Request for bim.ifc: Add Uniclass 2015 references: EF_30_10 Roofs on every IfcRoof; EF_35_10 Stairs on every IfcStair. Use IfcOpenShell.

First a look at what the model holds.

```python
import ifcopenshell

model = ifcopenshell.open("bim.ifc")
print(model.schema)
print("classifications:", [c.Name for c in model.by_type("IfcClassification")])
for ifc_class in ("IfcDoor", "IfcRoof", "IfcStair", "IfcWall", "IfcWindow"):
    print(ifc_class, len(model.by_type(ifc_class)))
```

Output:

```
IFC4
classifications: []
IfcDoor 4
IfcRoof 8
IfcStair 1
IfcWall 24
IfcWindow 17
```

```python
import ifcopenshell
import ifcopenshell.api.classification

model = ifcopenshell.open("bim.ifc")

system = ifcopenshell.api.classification.add_classification(model, classification="Uniclass 2015")

codes = {
    "IfcRoof": ("EF_30_10", "Roofs"),
    "IfcStair": ("EF_35_10", "Stairs"),
}
for ifc_class, (code, name) in codes.items():
    products = model.by_type(ifc_class)
    ifcopenshell.api.classification.add_reference(
        model, products=products, classification=system, identification=code, name=name
    )
    print(code, len(products))

model.write("bim_v2.ifc")
```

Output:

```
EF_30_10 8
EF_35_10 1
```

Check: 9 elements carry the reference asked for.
